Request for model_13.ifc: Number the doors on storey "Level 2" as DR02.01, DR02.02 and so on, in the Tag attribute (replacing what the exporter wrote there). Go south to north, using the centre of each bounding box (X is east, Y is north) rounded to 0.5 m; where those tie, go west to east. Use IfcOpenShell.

First a look at what the model holds.

```python
import ifcopenshell
import ifcopenshell.util.element
import ifcopenshell.util.placement

model = ifcopenshell.open("model_13.ifc")
print(model.schema)
storey = next(s for s in model.by_type("IfcBuildingStorey") if s.Name == "Level 2")
doors = [e for e in ifcopenshell.util.element.get_decomposition(storey) if e.is_a("IfcDoor")]
for e in sorted(doors, key=lambda e: e.id()):
    origin = ifcopenshell.util.placement.get_local_placement(e.ObjectPlacement)[:3, 3]
    print(e.id(), e.Tag, e.Name, origin.round(2) + 0.0, sep=" | ")
```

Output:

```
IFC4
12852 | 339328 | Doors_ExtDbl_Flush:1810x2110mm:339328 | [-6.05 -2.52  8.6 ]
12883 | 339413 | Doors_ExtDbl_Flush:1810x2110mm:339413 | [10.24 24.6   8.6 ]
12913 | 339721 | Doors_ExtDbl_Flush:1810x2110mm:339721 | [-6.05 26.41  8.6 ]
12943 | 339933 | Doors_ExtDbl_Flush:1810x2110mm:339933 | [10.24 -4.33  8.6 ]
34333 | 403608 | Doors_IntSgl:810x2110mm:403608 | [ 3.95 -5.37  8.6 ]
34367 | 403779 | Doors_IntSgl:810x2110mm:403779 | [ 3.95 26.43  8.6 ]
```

```python
import ifcopenshell
import ifcopenshell.geom
import ifcopenshell.util.element
import ifcopenshell.util.shape

model = ifcopenshell.open("model_13.ifc")
settings = ifcopenshell.geom.settings()
settings.set("use-world-coords", True)


def centre(element):
    shape = ifcopenshell.geom.create_shape(settings, element)
    return ifcopenshell.util.shape.get_bbox_centroid(shape.geometry)


storey = next(s for s in model.by_type("IfcBuildingStorey") if s.Name == "Level 2")
doors = [e for e in ifcopenshell.util.element.get_decomposition(storey) if e.is_a("IfcDoor")]

# Insertion points can sit at a corner or the storey origin, so sort by the geometry (in metres).
centres = {e: centre(e) for e in doors}
doors.sort(key=lambda e: (round(centres[e][1] / 0.5), centres[e][0]))

for i, e in enumerate(doors, start=1):
    number = f"DR02.{i:02d}"
    e.Tag = number
    print(e.id(), number)

model.write("model_13_rev.ifc")
```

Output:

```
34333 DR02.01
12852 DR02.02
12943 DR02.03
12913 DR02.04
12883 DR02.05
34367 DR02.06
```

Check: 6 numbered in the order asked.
